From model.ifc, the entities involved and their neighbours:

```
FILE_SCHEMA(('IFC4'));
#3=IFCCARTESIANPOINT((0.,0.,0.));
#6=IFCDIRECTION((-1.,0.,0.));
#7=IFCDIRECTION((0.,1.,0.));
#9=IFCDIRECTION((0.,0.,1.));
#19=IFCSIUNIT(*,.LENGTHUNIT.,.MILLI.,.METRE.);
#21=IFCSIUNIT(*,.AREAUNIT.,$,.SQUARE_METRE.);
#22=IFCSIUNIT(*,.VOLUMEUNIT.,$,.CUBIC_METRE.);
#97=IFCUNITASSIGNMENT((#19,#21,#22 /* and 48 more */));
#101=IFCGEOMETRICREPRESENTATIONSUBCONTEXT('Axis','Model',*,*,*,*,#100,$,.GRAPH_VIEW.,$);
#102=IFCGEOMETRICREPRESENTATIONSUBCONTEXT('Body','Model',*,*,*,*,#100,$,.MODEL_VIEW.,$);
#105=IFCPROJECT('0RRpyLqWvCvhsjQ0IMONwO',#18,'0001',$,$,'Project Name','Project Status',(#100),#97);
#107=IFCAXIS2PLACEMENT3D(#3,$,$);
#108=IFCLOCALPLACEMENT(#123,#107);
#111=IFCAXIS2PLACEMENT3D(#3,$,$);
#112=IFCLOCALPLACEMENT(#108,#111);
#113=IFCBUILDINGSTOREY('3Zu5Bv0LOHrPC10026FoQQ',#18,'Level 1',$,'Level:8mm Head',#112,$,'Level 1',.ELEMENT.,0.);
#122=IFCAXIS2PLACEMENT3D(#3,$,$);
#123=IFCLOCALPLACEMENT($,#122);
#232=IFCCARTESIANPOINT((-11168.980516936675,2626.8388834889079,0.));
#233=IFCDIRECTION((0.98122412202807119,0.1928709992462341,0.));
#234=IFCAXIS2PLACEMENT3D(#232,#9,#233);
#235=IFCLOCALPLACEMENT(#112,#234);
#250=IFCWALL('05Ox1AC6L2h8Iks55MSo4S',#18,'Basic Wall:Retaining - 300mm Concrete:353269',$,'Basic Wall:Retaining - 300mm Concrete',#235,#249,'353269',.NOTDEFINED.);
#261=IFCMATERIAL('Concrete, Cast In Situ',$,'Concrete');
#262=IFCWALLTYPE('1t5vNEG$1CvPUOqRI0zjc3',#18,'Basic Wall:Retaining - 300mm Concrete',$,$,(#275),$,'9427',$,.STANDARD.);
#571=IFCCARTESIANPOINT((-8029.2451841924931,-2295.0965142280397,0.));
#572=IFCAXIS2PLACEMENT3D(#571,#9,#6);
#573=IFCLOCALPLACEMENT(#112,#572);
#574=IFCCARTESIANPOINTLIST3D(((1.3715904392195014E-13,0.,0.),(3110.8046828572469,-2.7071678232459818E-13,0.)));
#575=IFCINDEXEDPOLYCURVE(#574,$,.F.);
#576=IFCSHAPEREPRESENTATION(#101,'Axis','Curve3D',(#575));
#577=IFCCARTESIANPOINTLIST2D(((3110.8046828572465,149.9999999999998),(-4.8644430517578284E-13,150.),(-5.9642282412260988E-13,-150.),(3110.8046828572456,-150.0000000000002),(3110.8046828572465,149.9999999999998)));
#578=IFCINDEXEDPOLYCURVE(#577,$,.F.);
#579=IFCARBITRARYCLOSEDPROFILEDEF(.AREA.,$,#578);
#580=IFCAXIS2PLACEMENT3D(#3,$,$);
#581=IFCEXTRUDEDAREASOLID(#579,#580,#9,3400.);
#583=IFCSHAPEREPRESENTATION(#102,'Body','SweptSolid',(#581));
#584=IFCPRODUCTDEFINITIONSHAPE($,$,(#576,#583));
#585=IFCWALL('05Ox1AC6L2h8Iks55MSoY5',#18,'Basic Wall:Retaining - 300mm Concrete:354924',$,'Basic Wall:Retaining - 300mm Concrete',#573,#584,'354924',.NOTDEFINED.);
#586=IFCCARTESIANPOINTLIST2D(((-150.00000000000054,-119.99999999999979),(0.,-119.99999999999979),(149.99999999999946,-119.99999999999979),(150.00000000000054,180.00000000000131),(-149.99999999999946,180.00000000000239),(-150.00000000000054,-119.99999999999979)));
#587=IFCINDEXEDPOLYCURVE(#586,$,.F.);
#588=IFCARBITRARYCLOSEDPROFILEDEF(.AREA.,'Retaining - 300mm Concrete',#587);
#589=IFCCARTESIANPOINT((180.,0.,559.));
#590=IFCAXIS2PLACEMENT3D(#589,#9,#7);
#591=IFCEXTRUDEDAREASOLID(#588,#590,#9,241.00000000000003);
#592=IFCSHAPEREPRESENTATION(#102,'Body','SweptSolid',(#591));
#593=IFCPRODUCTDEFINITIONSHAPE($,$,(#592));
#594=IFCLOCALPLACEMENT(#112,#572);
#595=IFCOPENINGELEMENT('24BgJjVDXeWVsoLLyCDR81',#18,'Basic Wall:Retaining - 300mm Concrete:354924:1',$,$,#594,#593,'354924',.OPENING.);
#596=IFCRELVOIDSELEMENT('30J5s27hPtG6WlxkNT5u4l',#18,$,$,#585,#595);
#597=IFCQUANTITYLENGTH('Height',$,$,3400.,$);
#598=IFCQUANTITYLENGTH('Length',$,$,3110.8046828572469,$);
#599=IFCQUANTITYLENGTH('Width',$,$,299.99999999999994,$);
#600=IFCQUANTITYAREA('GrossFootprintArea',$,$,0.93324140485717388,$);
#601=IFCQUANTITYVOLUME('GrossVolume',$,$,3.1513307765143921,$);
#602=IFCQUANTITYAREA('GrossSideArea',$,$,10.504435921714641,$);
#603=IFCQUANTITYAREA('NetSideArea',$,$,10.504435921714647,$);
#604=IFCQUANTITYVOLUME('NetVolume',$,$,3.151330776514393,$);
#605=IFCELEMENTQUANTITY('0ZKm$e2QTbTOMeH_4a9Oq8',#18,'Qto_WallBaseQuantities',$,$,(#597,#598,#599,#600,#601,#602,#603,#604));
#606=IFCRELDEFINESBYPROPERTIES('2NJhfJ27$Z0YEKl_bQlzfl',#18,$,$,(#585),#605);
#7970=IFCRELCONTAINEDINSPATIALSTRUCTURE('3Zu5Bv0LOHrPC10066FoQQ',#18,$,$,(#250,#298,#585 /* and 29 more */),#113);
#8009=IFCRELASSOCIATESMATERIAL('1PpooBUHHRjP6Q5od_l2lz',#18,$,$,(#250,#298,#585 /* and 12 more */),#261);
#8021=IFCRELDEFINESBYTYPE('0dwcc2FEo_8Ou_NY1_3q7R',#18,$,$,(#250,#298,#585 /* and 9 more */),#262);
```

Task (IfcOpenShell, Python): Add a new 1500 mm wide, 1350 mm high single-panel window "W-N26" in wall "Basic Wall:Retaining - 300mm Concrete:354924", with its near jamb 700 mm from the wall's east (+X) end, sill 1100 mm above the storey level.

```python
import numpy as np
import ifcopenshell
import ifcopenshell.api.feature
import ifcopenshell.api.geometry
import ifcopenshell.api.pset
import ifcopenshell.api.root
import ifcopenshell.api.spatial
import ifcopenshell.geom
import ifcopenshell.util.element
import ifcopenshell.util.placement
import ifcopenshell.util.representation
import ifcopenshell.util.shape
import ifcopenshell.util.unit

model = ifcopenshell.open("model.ifc")
unit_scale = ifcopenshell.util.unit.calculate_unit_scale(model)
area_scale = ifcopenshell.util.unit.calculate_unit_scale(model, "AREAUNIT")
volume_scale = ifcopenshell.util.unit.calculate_unit_scale(model, "VOLUMEUNIT")
settings = ifcopenshell.geom.settings()


def volume(element):
    """Net volume in cubic metres, openings subtracted."""
    shape = ifcopenshell.geom.create_shape(settings, element)
    return ifcopenshell.util.shape.get_volume(shape.geometry)


wall = model.by_guid("05Ox1AC6L2h8Iks55MSoY5")
storey = ifcopenshell.util.element.get_container(wall, ifc_class="IfcBuildingStorey")
context = ifcopenshell.util.representation.get_context(model, "Model", "Body", "MODEL_VIEW")
before = volume(wall)

width, height, from_end, sill = 1.5, 1.35, 0.7, 1.1  # metres

# The wall runs along its own X axis, and the end named is its -X end.
wall_shape = ifcopenshell.geom.create_shape(settings, wall)
x, y, z = ifcopenshell.util.shape.get_vertices(wall_shape.geometry).T
start = x.min() + from_end
face, thickness = float(y.min()), float(y.max() - y.min())
wall_matrix = ifcopenshell.util.placement.get_local_placement(wall.ObjectPlacement)
level = ifcopenshell.util.placement.get_local_placement(storey.ObjectPlacement)[2, 3]


def in_wall(x, y):
    """Placement at x, y metres in the wall's axes, at sill height."""
    matrix = wall_matrix.copy()
    matrix[:, 3] = wall_matrix @ np.array([x / unit_scale, y / unit_scale, 0.0, 1.0])
    matrix[2, 3] = level + sill / unit_scale
    return matrix


# Opening: a box that overshoots both wall faces by 50 mm.
opening = ifcopenshell.api.root.create_entity(model, ifc_class="IfcOpeningElement", predefined_type="OPENING")
box = ifcopenshell.api.geometry.add_wall_representation(
    model, context=context, length=width, height=height, thickness=thickness + 0.1
)
ifcopenshell.api.geometry.assign_representation(model, product=opening, representation=box)
ifcopenshell.api.geometry.edit_object_placement(model, product=opening, matrix=in_wall(start, face - 0.05), is_si=False)
ifcopenshell.api.feature.add_feature(model, feature=opening, element=wall)

window = ifcopenshell.api.root.create_entity(model, ifc_class="IfcWindow", name="W-N26", predefined_type="WINDOW")
window.OverallWidth, window.OverallHeight = width / unit_scale, height / unit_scale
window.PartitioningType = "SINGLE_PANEL"
body = ifcopenshell.api.geometry.add_window_representation(
    model,
    context=context,
    overall_width=window.OverallWidth,
    overall_height=window.OverallHeight,
    partition_type="SINGLE_PANEL",
)
ifcopenshell.api.geometry.assign_representation(model, product=window, representation=body)
ifcopenshell.api.spatial.assign_container(model, products=[window], relating_structure=storey)
ifcopenshell.api.feature.add_filling(model, opening=opening, element=window)

# Centre the window in the wall's thickness.
ifcopenshell.api.geometry.edit_object_placement(model, product=window, matrix=in_wall(start, face), is_si=False)
window_shape = ifcopenshell.geom.create_shape(settings, window)
depth = ifcopenshell.util.shape.get_vertices(window_shape.geometry)[:, 1]
offset = face + thickness / 2 - (depth.min() + depth.max()) / 2
ifcopenshell.api.geometry.edit_object_placement(model, product=window, matrix=in_wall(start, offset), is_si=False)

after = volume(wall)

# Update the wall's stored quantities.
qto = model.by_id(ifcopenshell.util.element.get_pset(wall, "Qto_WallBaseQuantities", should_inherit=False)["id"])
ifcopenshell.api.pset.edit_qto(model, qto=qto, properties={
    "NetSideArea": after / thickness / area_scale,
    "NetVolume": after / volume_scale,
})

print(f"wall volume {before:.3f} -> {after:.3f} m3")

model.write("model_v2.ifc")
```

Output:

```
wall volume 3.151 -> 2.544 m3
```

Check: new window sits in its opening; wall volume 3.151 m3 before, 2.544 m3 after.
